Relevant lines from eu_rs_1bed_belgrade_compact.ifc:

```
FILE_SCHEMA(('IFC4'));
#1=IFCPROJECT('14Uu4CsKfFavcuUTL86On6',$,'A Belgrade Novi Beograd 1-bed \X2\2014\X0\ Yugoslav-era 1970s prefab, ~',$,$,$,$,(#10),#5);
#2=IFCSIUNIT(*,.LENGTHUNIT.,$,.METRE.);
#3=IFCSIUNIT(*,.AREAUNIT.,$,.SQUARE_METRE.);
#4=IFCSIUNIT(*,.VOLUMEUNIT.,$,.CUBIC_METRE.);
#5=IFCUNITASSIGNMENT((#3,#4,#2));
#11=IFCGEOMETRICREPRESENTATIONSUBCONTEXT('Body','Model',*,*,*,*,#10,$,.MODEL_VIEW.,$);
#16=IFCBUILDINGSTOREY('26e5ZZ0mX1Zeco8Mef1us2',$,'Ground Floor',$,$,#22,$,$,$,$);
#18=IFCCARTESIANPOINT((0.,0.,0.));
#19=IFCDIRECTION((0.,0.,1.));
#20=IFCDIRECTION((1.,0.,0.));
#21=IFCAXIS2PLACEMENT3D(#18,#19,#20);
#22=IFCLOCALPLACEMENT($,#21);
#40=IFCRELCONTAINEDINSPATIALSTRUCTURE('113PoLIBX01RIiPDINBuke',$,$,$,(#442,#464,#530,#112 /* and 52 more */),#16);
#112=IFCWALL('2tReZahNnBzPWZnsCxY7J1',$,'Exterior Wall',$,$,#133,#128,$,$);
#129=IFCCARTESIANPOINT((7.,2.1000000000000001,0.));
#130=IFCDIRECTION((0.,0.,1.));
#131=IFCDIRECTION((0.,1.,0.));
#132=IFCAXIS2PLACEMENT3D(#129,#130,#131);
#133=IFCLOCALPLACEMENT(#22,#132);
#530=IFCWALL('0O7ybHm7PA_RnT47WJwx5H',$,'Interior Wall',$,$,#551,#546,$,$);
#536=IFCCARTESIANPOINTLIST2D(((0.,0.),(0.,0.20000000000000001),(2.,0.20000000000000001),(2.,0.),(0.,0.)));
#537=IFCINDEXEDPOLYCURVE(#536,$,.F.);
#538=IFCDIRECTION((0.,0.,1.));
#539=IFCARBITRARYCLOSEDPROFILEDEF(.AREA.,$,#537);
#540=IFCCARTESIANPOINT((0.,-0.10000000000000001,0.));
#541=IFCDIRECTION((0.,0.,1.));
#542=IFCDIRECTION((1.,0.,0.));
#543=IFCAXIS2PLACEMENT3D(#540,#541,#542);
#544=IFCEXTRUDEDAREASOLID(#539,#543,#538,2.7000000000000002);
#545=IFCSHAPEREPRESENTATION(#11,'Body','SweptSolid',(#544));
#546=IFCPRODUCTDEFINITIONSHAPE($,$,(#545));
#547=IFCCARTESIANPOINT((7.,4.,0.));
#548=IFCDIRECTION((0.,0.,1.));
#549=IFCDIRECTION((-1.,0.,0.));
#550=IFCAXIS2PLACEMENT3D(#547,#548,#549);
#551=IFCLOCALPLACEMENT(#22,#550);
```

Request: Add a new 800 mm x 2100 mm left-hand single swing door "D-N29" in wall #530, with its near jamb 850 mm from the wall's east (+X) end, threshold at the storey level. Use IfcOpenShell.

```python
import numpy as np
import ifcopenshell
import ifcopenshell.api.feature
import ifcopenshell.api.geometry
import ifcopenshell.api.root
import ifcopenshell.api.spatial
import ifcopenshell.geom
import ifcopenshell.util.element
import ifcopenshell.util.placement
import ifcopenshell.util.representation
import ifcopenshell.util.shape
import ifcopenshell.util.unit

model = ifcopenshell.open("eu_rs_1bed_belgrade_compact.ifc")
unit_scale = ifcopenshell.util.unit.calculate_unit_scale(model)
settings = ifcopenshell.geom.settings()


def volume(element):
    """Net volume in cubic metres, openings subtracted."""
    shape = ifcopenshell.geom.create_shape(settings, element)
    return ifcopenshell.util.shape.get_volume(shape.geometry)


wall = model.by_guid("0O7ybHm7PA_RnT47WJwx5H")
storey = ifcopenshell.util.element.get_container(wall, ifc_class="IfcBuildingStorey")
context = ifcopenshell.util.representation.get_context(model, "Model", "Body", "MODEL_VIEW")
before = volume(wall)

width, height, from_end, sill = 0.8, 2.1, 0.85, 0.0  # metres

# The wall runs along its own X axis, and the end named is its -X end.
wall_shape = ifcopenshell.geom.create_shape(settings, wall)
x, y, z = ifcopenshell.util.shape.get_vertices(wall_shape.geometry).T
start = x.min() + from_end
face, thickness = float(y.min()), float(y.max() - y.min())
wall_matrix = ifcopenshell.util.placement.get_local_placement(wall.ObjectPlacement)
level = ifcopenshell.util.placement.get_local_placement(storey.ObjectPlacement)[2, 3]


def in_wall(x, y):
    """Placement at x, y metres in the wall's axes, at sill height."""
    matrix = wall_matrix.copy()
    matrix[:, 3] = wall_matrix @ np.array([x / unit_scale, y / unit_scale, 0.0, 1.0])
    matrix[2, 3] = level + sill / unit_scale
    return matrix


# Opening: a box that overshoots both wall faces by 50 mm.
opening = ifcopenshell.api.root.create_entity(model, ifc_class="IfcOpeningElement", predefined_type="OPENING")
box = ifcopenshell.api.geometry.add_wall_representation(
    model, context=context, length=width, height=height, thickness=thickness + 0.1
)
ifcopenshell.api.geometry.assign_representation(model, product=opening, representation=box)
ifcopenshell.api.geometry.edit_object_placement(model, product=opening, matrix=in_wall(start, face - 0.05), is_si=False)
ifcopenshell.api.feature.add_feature(model, feature=opening, element=wall)

door = ifcopenshell.api.root.create_entity(model, ifc_class="IfcDoor", name="D-N29", predefined_type="DOOR")
door.OverallWidth, door.OverallHeight = width / unit_scale, height / unit_scale
door.OperationType = "SINGLE_SWING_LEFT"
body = ifcopenshell.api.geometry.add_door_representation(
    model,
    context=context,
    overall_width=door.OverallWidth,
    overall_height=door.OverallHeight,
    operation_type="SINGLE_SWING_LEFT",
    lining_properties={"LiningDepth": thickness / unit_scale, "ThresholdDepth": thickness / unit_scale},
)
ifcopenshell.api.geometry.assign_representation(model, product=door, representation=body)
ifcopenshell.api.spatial.assign_container(model, products=[door], relating_structure=storey)
ifcopenshell.api.feature.add_filling(model, opening=opening, element=door)

# The lining spans the wall, so the door starts at the wall face.
ifcopenshell.api.geometry.edit_object_placement(model, product=door, matrix=in_wall(start, face), is_si=False)

after = volume(wall)

print(f"wall volume {before:.3f} -> {after:.3f} m3")

model.write("eu_rs_1bed_belgrade_compact_updated.ifc")
```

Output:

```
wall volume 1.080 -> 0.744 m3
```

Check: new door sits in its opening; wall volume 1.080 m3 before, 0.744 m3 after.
